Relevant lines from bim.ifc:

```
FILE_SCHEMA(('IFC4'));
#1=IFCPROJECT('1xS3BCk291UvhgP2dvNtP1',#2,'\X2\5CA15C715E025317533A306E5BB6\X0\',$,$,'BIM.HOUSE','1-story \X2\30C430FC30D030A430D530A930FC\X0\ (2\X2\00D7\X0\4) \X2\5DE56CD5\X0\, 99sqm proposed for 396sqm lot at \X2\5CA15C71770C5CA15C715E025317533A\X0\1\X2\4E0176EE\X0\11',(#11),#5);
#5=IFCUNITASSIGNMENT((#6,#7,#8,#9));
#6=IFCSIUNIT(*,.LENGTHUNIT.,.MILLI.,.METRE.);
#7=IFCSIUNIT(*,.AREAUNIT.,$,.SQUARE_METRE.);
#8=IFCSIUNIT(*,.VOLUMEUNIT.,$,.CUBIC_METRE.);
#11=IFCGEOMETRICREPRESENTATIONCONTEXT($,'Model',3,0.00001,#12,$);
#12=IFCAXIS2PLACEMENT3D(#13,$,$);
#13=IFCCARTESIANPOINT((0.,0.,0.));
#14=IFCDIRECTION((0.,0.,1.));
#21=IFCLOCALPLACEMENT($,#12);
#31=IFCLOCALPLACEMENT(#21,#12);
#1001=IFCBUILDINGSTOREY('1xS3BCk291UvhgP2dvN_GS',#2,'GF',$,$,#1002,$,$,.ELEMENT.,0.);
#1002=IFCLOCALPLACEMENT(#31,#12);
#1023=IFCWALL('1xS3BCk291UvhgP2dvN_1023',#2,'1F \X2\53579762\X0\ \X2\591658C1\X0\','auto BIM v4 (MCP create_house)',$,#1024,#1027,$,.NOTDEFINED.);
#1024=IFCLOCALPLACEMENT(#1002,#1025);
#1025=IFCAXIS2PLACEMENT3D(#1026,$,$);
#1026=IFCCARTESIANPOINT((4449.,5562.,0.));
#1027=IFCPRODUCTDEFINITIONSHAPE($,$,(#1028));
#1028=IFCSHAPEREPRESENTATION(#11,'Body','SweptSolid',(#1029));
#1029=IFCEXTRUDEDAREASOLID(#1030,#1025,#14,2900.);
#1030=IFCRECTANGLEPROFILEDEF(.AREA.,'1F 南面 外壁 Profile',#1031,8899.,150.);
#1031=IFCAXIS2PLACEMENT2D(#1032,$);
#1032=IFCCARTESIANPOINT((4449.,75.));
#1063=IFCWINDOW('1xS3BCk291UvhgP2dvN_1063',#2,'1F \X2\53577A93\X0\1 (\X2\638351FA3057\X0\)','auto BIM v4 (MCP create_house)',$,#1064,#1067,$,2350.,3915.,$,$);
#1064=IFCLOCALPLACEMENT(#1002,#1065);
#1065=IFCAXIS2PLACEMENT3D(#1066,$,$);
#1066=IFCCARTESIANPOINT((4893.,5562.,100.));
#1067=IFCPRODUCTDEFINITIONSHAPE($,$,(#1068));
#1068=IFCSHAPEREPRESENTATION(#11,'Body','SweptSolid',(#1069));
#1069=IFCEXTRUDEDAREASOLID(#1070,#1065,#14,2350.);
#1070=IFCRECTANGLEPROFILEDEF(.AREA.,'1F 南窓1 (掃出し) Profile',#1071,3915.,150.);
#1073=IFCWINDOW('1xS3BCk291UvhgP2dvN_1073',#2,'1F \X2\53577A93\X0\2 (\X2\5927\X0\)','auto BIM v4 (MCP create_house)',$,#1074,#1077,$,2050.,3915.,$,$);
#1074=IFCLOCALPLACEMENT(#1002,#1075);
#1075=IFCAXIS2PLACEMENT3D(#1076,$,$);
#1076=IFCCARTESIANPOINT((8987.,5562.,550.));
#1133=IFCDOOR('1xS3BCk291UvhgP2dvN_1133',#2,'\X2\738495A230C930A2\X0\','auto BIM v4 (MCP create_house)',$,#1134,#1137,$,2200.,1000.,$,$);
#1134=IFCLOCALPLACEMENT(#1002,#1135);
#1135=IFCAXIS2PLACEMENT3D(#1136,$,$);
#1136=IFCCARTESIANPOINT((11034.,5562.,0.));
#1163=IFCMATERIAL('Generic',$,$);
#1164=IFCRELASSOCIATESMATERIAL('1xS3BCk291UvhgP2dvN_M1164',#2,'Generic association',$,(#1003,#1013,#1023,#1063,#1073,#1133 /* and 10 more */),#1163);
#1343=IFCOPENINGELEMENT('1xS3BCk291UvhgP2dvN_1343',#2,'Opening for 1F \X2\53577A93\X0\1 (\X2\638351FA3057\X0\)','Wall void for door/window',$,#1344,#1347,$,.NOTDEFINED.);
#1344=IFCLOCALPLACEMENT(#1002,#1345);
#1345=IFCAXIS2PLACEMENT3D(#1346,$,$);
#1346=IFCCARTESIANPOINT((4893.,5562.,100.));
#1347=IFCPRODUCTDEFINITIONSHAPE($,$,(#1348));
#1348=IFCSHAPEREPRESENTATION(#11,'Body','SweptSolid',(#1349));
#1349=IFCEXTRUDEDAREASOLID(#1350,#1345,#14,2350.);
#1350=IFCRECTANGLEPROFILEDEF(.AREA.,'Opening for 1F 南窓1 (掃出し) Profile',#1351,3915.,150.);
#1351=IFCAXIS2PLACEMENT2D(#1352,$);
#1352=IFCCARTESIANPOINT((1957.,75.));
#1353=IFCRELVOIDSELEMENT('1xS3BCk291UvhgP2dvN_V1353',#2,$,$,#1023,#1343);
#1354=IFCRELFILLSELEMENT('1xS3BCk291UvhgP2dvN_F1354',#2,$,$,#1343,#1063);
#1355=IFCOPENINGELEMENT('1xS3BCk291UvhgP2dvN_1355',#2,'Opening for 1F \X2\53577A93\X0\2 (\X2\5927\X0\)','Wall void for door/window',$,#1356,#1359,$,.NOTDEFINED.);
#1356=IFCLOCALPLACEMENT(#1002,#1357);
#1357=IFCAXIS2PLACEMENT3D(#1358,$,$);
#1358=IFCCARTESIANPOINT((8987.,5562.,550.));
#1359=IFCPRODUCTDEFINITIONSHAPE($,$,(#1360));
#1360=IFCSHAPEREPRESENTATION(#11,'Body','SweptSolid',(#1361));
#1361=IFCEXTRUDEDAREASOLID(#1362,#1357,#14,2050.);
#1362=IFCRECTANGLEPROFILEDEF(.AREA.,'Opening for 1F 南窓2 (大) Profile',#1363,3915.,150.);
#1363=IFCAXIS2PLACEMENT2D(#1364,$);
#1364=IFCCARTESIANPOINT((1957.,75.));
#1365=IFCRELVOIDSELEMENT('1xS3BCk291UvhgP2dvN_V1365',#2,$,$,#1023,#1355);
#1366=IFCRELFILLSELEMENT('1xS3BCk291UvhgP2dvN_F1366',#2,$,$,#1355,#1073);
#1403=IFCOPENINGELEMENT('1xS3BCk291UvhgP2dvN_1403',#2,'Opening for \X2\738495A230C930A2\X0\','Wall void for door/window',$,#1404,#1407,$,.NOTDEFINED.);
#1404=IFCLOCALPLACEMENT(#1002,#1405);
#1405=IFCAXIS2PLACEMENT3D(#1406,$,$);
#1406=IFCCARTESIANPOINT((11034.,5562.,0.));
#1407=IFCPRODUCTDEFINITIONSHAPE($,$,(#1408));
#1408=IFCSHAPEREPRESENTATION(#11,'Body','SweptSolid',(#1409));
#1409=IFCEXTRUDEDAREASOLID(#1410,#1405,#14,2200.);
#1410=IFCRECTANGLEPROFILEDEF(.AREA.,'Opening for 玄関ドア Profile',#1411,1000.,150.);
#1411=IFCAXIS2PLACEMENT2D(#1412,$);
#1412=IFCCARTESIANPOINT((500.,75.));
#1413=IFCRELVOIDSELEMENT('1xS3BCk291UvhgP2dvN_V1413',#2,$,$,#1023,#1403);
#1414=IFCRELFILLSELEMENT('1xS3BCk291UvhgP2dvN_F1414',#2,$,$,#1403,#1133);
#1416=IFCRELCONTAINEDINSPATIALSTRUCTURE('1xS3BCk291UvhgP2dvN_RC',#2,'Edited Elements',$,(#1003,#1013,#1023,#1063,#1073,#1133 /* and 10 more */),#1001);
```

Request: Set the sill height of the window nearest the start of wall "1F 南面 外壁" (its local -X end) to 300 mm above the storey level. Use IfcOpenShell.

```python
import numpy as np
import ifcopenshell
import ifcopenshell.api.geometry
import ifcopenshell.geom
import ifcopenshell.util.element
import ifcopenshell.util.placement
import ifcopenshell.util.shape
import ifcopenshell.util.unit

model = ifcopenshell.open("bim.ifc")
unit_scale = ifcopenshell.util.unit.calculate_unit_scale(model)

window = model.by_id(1063)
opening = window.FillsVoids[0].RelatingOpeningElement
storey = ifcopenshell.util.element.get_container(window, ifc_class="IfcBuildingStorey")
level = ifcopenshell.util.placement.get_local_placement(storey.ObjectPlacement)[2, 3]

# The opening's origin need not be at the sill, so measure its lowest point.
shape = ifcopenshell.geom.create_shape(ifcopenshell.geom.settings(), opening)
bottom = ifcopenshell.util.shape.get_shape_bottom_elevation(shape, shape.geometry) / unit_scale
dz = level + 300.0 - bottom

shift = np.array([0.0, 0.0, dz])
# The window is not placed relative to its opening, so move both.
for product in (opening, window):
    matrix = ifcopenshell.util.placement.get_local_placement(product.ObjectPlacement)
    matrix[:3, 3] += shift
    ifcopenshell.api.geometry.edit_object_placement(model, product=product, matrix=matrix, is_si=False)

print(f"moved by {dz * unit_scale:+.3f} m")

model.write("bim_rev.ifc")
```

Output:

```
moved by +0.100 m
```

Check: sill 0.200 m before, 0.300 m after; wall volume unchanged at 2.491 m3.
